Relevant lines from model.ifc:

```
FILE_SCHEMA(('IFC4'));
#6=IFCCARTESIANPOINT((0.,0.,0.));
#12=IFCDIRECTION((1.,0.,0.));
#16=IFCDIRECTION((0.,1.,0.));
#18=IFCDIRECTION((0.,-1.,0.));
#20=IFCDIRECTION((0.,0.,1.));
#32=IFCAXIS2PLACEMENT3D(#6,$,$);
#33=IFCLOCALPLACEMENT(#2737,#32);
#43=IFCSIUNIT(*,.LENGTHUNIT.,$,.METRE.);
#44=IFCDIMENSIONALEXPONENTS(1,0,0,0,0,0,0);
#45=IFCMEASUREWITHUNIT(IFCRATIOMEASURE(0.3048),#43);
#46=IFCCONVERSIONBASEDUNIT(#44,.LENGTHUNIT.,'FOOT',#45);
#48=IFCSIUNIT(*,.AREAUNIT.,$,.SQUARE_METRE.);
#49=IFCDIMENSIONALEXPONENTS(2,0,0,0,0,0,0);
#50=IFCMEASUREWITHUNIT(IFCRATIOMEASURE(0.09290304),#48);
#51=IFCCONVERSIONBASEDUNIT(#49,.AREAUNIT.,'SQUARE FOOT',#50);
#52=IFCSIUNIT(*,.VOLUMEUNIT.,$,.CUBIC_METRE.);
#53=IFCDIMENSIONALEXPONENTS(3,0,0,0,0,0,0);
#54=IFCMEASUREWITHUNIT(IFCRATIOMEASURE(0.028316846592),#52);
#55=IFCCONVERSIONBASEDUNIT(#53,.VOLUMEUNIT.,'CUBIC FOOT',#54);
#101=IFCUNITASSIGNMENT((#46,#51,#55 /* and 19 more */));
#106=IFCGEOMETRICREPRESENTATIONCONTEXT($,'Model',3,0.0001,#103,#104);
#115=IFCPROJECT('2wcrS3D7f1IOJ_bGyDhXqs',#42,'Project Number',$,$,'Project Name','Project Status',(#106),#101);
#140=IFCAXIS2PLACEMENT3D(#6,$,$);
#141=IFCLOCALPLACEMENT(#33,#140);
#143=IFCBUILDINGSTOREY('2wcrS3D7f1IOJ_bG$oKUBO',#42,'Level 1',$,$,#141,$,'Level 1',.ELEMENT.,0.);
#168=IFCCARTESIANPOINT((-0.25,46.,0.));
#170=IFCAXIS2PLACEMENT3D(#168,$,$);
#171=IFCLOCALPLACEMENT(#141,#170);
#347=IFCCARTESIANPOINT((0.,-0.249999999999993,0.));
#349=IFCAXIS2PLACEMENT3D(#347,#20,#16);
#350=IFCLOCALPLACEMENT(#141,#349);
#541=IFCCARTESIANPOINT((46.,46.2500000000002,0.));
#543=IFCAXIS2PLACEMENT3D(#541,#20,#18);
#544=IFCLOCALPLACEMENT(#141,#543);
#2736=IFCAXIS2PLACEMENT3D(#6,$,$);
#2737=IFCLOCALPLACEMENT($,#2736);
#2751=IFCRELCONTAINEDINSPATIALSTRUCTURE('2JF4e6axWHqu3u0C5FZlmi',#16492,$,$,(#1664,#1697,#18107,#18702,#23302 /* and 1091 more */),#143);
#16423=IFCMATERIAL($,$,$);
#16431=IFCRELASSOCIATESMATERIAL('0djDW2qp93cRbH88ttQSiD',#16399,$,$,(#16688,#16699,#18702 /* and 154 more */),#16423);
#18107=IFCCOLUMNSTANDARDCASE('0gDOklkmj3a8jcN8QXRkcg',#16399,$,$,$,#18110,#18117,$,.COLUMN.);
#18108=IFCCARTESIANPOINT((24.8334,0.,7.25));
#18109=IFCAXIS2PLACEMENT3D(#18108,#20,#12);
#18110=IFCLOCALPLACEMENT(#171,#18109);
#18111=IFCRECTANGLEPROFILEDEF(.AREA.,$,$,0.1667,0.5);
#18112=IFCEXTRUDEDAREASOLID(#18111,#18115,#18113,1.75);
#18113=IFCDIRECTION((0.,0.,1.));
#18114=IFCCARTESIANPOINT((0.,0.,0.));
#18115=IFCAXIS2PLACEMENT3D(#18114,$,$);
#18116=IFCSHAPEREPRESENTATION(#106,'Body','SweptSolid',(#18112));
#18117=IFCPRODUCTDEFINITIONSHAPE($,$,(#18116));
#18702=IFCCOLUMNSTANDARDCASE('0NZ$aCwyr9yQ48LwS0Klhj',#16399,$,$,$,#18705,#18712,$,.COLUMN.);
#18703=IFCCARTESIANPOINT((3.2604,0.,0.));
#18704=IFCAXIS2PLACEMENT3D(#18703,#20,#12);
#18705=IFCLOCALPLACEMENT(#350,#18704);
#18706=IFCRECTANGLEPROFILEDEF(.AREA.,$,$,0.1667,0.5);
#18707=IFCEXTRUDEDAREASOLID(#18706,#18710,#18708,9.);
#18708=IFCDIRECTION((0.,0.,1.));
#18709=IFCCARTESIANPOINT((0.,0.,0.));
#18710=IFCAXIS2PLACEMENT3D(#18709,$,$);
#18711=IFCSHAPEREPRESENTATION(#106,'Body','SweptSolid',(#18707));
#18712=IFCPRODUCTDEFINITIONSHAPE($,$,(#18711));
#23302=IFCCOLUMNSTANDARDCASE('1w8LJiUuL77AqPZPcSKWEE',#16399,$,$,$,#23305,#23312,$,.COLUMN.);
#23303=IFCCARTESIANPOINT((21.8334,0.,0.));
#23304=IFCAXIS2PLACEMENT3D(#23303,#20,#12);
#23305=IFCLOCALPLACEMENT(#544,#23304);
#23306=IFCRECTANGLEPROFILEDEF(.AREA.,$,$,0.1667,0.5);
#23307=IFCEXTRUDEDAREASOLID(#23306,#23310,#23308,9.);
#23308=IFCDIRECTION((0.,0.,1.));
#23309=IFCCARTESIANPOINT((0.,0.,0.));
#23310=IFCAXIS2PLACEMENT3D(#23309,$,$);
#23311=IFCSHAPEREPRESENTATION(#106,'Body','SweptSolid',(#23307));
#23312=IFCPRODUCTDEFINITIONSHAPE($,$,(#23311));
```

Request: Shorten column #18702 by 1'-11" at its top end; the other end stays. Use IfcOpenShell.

```python
import ifcopenshell
import ifcopenshell.util.unit

model = ifcopenshell.open("model.ifc")
unit_scale = ifcopenshell.util.unit.calculate_unit_scale(model)

member = model.by_guid("0NZ$aCwyr9yQ48LwS0Klhj")
change = -23 * 0.0254 / unit_scale

# The extrusion runs towards the end named, so only its depth changes.
body = next(r for r in member.Representation.Representations if r.RepresentationIdentifier == "Body")
solid = body.Items[0]
old_length = solid.Depth
solid.Depth += change

print(f"length {old_length:g} -> {solid.Depth:g}")

model.write("model_v2.ifc")
```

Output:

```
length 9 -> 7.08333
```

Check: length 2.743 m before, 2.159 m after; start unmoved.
